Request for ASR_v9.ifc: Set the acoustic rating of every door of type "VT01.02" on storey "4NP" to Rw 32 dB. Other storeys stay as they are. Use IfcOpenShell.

First a look at what the model holds.

```python
import ifcopenshell
import ifcopenshell.util.element

model = ifcopenshell.open("ASR_v9.ifc")
print(model.schema)
storey = next(s for s in model.by_type("IfcBuildingStorey") if s.Name == "4NP")
doors = [e for e in ifcopenshell.util.element.get_decomposition(storey) if e.is_a("IfcDoor")]
seen = {}
for e in doors:
    element_type = ifcopenshell.util.element.get_type(e)
    key = (element_type.Name if element_type != e and element_type else None, ifcopenshell.util.element.get_pset(e, "Pset_DoorCommon", "AcousticRating"))
    seen[key] = seen.get(key, 0) + 1
for (name, value), count in sorted(seen.items(), key=str):
    print(count, "x", name, "|", value)
```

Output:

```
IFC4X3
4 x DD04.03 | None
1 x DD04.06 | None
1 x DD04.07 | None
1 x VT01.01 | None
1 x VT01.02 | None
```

```python
import ifcopenshell
import ifcopenshell.api.pset
import ifcopenshell.util.element

model = ifcopenshell.open("ASR_v9.ifc")

storey = next(s for s in model.by_type("IfcBuildingStorey") if s.Name == "4NP")
doors = [e for e in ifcopenshell.util.element.get_decomposition(storey) if e.is_a("IfcDoor")]

count = 0
for e in doors:
    element_type = ifcopenshell.util.element.get_type(e)
    if element_type in (None, e) or element_type.Name != "VT01.02":
        continue
    # add_pset returns the element's existing set when there is one.
    pset = ifcopenshell.api.pset.add_pset(model, product=e, name="Pset_DoorCommon")
    ifcopenshell.api.pset.edit_pset(model, pset=pset, properties={"AcousticRating": "Rw 32 dB"})
    count += 1

print(count, "doors updated")

model.write("ASR_v9_v2.ifc")
```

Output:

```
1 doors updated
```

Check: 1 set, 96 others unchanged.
